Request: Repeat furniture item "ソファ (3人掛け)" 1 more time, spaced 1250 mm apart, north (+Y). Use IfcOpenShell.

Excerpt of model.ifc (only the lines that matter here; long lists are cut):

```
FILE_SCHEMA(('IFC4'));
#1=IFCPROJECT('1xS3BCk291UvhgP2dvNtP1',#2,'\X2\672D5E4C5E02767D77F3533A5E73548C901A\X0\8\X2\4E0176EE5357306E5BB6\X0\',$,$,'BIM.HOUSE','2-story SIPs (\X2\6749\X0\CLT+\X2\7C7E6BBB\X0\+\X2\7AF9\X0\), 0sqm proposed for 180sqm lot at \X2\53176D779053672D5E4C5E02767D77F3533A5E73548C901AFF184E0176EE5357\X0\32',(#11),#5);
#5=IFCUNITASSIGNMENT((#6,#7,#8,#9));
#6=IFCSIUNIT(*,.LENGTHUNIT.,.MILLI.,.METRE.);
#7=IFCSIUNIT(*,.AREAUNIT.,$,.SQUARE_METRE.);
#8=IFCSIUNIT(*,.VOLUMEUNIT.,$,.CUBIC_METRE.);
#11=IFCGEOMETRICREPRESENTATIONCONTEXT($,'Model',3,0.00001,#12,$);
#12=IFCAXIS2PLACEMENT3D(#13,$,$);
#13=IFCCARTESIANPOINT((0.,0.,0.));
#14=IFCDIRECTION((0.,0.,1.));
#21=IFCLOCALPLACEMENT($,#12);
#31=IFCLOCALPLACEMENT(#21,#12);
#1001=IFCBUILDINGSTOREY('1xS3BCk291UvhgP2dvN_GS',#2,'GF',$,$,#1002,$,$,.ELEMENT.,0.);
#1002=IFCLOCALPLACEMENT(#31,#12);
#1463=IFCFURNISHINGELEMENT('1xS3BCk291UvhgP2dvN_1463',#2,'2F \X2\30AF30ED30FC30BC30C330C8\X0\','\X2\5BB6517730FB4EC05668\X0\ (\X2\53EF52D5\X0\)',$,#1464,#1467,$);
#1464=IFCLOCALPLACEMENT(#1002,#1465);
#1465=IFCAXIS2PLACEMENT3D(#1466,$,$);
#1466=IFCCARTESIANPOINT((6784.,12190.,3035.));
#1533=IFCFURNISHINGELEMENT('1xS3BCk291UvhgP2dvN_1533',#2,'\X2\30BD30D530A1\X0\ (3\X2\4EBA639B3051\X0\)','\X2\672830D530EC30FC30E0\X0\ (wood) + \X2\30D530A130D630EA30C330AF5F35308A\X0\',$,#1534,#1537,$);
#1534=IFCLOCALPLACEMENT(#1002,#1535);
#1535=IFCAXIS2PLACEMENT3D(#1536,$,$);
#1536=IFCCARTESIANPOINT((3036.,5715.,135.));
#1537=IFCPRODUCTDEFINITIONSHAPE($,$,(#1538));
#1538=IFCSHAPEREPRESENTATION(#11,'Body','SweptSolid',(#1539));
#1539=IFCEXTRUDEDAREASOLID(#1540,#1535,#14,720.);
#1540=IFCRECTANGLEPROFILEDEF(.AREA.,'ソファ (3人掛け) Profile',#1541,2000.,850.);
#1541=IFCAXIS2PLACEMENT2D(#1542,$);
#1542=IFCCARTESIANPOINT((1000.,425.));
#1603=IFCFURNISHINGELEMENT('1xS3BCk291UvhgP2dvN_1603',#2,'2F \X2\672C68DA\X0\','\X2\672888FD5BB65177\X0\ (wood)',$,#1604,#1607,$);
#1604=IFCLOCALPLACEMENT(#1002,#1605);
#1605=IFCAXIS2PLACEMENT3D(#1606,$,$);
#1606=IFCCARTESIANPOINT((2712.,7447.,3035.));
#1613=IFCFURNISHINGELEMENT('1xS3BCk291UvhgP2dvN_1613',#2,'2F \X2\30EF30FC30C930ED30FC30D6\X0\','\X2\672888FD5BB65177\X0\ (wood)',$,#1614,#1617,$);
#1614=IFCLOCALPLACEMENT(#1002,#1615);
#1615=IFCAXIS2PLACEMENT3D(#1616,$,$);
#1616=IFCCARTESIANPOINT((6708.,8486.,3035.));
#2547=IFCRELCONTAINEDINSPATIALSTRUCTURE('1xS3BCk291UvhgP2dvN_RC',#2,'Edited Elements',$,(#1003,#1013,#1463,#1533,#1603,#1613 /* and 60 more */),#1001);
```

```python
import numpy as np
import ifcopenshell
import ifcopenshell.api.geometry
import ifcopenshell.api.root
import ifcopenshell.util.element
import ifcopenshell.util.placement

model = ifcopenshell.open("model.ifc")


def reuse_history(source, copy):
    """copy_class also copies each property set's owner history, people and application; keep the originals."""
    for rel in copy.IsDefinedBy:
        if rel.is_a("IfcRelDefinesByProperties") and (history := rel.RelatingPropertyDefinition.OwnerHistory):
            rel.RelatingPropertyDefinition.OwnerHistory = source.OwnerHistory
            ifcopenshell.util.element.remove_deep2(model, history)


source = model.by_guid("1xS3BCk291UvhgP2dvN_1533")
base = ifcopenshell.util.placement.get_local_placement(source.ObjectPlacement)
step = np.array([0.0, 1.0, 0.0]) * 1250.0

for i in range(1, 2):
    copy = ifcopenshell.api.root.copy_class(model, product=source)
    copy.Representation = ifcopenshell.util.element.copy_deep(
        model, source.Representation, exclude=["IfcGeometricRepresentationContext", "IfcRepresentationMap"]
    )
    reuse_history(source, copy)
    matrix = base.copy()
    matrix[:3, 3] += i * step
    print("added at", matrix[:3, 3].round(3) + 0.0)
    ifcopenshell.api.geometry.edit_object_placement(model, product=copy, matrix=matrix, is_si=False)

model.write("model_v2.ifc")
```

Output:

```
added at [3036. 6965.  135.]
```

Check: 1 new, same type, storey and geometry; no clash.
